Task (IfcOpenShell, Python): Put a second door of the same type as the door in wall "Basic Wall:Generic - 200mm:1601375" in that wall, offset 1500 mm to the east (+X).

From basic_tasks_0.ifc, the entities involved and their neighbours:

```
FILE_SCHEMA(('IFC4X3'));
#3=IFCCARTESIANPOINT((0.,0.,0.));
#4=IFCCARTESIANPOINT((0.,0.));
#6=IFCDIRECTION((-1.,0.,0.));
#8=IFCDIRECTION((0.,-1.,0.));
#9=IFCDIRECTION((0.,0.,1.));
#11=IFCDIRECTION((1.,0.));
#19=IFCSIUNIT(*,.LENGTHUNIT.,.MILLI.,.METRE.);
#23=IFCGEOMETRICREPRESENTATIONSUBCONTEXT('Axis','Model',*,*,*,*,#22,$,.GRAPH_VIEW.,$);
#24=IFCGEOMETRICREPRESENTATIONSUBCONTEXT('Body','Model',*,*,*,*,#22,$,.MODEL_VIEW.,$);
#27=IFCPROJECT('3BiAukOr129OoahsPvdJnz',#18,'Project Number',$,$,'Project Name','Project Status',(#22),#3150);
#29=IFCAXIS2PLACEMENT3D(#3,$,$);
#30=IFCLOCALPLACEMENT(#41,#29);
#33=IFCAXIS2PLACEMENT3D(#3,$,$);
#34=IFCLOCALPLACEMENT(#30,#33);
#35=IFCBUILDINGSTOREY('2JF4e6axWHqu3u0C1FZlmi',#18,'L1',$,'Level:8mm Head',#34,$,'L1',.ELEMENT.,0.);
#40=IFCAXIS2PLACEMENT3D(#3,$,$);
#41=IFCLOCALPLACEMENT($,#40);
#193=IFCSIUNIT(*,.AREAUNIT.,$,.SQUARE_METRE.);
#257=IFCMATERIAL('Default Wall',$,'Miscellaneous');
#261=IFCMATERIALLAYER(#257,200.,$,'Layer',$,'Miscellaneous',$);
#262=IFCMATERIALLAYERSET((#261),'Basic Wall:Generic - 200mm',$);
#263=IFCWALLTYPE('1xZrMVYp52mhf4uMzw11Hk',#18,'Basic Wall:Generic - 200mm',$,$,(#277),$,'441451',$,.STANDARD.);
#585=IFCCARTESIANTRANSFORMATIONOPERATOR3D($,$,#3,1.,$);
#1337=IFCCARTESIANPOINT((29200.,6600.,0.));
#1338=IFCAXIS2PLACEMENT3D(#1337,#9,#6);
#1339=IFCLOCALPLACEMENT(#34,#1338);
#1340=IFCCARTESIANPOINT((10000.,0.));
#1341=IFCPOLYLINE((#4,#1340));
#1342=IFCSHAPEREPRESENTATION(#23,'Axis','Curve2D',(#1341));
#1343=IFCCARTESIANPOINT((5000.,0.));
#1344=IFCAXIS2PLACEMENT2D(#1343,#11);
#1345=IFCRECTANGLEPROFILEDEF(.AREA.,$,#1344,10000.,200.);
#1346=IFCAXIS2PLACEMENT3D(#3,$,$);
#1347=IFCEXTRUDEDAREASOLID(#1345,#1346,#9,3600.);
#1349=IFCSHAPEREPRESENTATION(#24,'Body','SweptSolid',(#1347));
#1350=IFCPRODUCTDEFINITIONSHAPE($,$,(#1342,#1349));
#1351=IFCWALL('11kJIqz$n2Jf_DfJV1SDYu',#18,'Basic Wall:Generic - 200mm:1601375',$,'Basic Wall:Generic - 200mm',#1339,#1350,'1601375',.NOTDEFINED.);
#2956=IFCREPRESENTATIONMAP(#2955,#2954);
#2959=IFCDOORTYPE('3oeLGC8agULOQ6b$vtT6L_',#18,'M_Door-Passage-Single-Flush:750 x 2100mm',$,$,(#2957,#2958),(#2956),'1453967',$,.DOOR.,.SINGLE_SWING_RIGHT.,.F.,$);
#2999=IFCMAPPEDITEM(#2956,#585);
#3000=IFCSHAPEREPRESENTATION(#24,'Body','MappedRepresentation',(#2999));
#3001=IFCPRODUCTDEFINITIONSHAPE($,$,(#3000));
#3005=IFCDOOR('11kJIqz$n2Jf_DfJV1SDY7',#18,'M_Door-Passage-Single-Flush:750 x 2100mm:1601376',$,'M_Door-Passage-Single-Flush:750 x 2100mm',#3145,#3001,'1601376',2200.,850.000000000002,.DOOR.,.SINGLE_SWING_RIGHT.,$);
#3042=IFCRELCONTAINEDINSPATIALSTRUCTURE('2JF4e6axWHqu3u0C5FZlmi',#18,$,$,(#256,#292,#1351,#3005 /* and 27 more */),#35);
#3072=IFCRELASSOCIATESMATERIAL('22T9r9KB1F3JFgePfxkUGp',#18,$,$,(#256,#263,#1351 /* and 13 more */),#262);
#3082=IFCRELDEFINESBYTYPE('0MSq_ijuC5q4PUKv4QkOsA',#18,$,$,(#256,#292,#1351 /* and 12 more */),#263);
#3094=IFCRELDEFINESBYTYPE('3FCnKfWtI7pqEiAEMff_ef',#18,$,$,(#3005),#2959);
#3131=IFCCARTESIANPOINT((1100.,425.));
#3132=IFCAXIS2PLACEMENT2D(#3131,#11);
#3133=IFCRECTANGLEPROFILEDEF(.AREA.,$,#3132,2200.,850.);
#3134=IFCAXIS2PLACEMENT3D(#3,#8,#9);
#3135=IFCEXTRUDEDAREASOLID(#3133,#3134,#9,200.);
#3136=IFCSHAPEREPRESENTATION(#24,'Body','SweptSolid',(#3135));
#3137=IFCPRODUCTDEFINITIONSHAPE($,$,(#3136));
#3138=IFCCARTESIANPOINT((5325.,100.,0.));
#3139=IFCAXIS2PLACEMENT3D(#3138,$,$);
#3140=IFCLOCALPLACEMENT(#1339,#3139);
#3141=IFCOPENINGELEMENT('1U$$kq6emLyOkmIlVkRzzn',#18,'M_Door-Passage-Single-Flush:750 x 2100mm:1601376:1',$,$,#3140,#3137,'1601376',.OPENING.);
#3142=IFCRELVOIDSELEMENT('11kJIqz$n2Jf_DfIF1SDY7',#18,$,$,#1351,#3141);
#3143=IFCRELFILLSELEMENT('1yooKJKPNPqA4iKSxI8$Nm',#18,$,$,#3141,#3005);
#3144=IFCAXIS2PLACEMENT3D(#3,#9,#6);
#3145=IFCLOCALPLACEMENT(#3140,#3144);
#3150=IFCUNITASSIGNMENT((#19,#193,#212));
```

```python
import ifcopenshell
import ifcopenshell.api.feature
import ifcopenshell.api.geometry
import ifcopenshell.api.root
import ifcopenshell.geom
import ifcopenshell.util.element
import ifcopenshell.util.placement
import ifcopenshell.util.shape
import ifcopenshell.util.unit

model = ifcopenshell.open("basic_tasks_0.ifc")
unit_scale = ifcopenshell.util.unit.calculate_unit_scale(model)
settings = ifcopenshell.geom.settings()


def volume(element):
    """Net volume in cubic metres, openings subtracted."""
    shape = ifcopenshell.geom.create_shape(settings, element)
    return ifcopenshell.util.shape.get_volume(shape.geometry)


def reuse_history(source, copy):
    """copy_class also copies each property set's owner history, people and application; keep the originals."""
    for rel in copy.IsDefinedBy:
        if rel.is_a("IfcRelDefinesByProperties") and (history := rel.RelatingPropertyDefinition.OwnerHistory):
            rel.RelatingPropertyDefinition.OwnerHistory = source.OwnerHistory
            ifcopenshell.util.element.remove_deep2(model, history)


door = model.by_id(3005)
opening = door.FillsVoids[0].RelatingOpeningElement
wall = opening.VoidsElements[0].RelatingBuildingElement
before = volume(wall)
shift = ifcopenshell.util.placement.get_local_placement(wall.ObjectPlacement)[:3, 0] * -1.5 / unit_scale

# copy_class copies the void relationship, type, container and properties, but no geometry.
new_opening = ifcopenshell.api.root.copy_class(model, product=opening)
new_opening.Representation = ifcopenshell.util.element.copy_deep(
    model, opening.Representation, exclude=["IfcGeometricRepresentationContext", "IfcRepresentationMap"]
)
new_opening.Name = "M_Door-Passage-Single-Flush:750 x 2100mm"
new_opening.Tag = None
new_door = ifcopenshell.api.root.copy_class(model, product=door)
new_door.Representation = ifcopenshell.util.element.copy_deep(
    model, door.Representation, exclude=["IfcGeometricRepresentationContext", "IfcRepresentationMap"]
)
new_door.Name = "M_Door-Passage-Single-Flush:750 x 2100mm"
new_door.Tag = None
reuse_history(door, new_door)
ifcopenshell.api.feature.add_filling(model, opening=new_opening, element=new_door)

for old, new in ((opening, new_opening), (door, new_door)):
    matrix = ifcopenshell.util.placement.get_local_placement(old.ObjectPlacement)
    matrix[:3, 3] += shift
    ifcopenshell.api.geometry.edit_object_placement(model, product=new, matrix=matrix, is_si=False)

after = volume(wall)

print(f"wall volume {before:.3f} -> {after:.3f} m3")

model.write("basic_tasks_0_updated.ifc")
```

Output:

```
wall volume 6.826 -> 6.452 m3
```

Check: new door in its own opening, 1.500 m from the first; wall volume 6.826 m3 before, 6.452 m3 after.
